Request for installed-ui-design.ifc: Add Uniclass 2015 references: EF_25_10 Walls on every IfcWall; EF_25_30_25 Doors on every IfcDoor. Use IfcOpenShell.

First a look at what the model holds.

```python
import ifcopenshell

model = ifcopenshell.open("installed-ui-design.ifc")
print(model.schema)
print("classifications:", [c.Name for c in model.by_type("IfcClassification")])
for ifc_class in ("IfcDoor", "IfcRoof", "IfcStair", "IfcWall", "IfcWindow"):
    print(ifc_class, len(model.by_type(ifc_class)))
```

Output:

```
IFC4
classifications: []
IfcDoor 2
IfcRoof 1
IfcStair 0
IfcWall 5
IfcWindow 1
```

```python
import ifcopenshell
import ifcopenshell.api.classification

model = ifcopenshell.open("installed-ui-design.ifc")

system = ifcopenshell.api.classification.add_classification(model, classification="Uniclass 2015")

codes = {
    "IfcWall": ("EF_25_10", "Walls"),
    "IfcDoor": ("EF_25_30_25", "Doors"),
}
for ifc_class, (code, name) in codes.items():
    products = model.by_type(ifc_class)
    ifcopenshell.api.classification.add_reference(
        model, products=products, classification=system, identification=code, name=name
    )
    print(code, len(products))

model.write("installed-ui-design_updated.ifc")
```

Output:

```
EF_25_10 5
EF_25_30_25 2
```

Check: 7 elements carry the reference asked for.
